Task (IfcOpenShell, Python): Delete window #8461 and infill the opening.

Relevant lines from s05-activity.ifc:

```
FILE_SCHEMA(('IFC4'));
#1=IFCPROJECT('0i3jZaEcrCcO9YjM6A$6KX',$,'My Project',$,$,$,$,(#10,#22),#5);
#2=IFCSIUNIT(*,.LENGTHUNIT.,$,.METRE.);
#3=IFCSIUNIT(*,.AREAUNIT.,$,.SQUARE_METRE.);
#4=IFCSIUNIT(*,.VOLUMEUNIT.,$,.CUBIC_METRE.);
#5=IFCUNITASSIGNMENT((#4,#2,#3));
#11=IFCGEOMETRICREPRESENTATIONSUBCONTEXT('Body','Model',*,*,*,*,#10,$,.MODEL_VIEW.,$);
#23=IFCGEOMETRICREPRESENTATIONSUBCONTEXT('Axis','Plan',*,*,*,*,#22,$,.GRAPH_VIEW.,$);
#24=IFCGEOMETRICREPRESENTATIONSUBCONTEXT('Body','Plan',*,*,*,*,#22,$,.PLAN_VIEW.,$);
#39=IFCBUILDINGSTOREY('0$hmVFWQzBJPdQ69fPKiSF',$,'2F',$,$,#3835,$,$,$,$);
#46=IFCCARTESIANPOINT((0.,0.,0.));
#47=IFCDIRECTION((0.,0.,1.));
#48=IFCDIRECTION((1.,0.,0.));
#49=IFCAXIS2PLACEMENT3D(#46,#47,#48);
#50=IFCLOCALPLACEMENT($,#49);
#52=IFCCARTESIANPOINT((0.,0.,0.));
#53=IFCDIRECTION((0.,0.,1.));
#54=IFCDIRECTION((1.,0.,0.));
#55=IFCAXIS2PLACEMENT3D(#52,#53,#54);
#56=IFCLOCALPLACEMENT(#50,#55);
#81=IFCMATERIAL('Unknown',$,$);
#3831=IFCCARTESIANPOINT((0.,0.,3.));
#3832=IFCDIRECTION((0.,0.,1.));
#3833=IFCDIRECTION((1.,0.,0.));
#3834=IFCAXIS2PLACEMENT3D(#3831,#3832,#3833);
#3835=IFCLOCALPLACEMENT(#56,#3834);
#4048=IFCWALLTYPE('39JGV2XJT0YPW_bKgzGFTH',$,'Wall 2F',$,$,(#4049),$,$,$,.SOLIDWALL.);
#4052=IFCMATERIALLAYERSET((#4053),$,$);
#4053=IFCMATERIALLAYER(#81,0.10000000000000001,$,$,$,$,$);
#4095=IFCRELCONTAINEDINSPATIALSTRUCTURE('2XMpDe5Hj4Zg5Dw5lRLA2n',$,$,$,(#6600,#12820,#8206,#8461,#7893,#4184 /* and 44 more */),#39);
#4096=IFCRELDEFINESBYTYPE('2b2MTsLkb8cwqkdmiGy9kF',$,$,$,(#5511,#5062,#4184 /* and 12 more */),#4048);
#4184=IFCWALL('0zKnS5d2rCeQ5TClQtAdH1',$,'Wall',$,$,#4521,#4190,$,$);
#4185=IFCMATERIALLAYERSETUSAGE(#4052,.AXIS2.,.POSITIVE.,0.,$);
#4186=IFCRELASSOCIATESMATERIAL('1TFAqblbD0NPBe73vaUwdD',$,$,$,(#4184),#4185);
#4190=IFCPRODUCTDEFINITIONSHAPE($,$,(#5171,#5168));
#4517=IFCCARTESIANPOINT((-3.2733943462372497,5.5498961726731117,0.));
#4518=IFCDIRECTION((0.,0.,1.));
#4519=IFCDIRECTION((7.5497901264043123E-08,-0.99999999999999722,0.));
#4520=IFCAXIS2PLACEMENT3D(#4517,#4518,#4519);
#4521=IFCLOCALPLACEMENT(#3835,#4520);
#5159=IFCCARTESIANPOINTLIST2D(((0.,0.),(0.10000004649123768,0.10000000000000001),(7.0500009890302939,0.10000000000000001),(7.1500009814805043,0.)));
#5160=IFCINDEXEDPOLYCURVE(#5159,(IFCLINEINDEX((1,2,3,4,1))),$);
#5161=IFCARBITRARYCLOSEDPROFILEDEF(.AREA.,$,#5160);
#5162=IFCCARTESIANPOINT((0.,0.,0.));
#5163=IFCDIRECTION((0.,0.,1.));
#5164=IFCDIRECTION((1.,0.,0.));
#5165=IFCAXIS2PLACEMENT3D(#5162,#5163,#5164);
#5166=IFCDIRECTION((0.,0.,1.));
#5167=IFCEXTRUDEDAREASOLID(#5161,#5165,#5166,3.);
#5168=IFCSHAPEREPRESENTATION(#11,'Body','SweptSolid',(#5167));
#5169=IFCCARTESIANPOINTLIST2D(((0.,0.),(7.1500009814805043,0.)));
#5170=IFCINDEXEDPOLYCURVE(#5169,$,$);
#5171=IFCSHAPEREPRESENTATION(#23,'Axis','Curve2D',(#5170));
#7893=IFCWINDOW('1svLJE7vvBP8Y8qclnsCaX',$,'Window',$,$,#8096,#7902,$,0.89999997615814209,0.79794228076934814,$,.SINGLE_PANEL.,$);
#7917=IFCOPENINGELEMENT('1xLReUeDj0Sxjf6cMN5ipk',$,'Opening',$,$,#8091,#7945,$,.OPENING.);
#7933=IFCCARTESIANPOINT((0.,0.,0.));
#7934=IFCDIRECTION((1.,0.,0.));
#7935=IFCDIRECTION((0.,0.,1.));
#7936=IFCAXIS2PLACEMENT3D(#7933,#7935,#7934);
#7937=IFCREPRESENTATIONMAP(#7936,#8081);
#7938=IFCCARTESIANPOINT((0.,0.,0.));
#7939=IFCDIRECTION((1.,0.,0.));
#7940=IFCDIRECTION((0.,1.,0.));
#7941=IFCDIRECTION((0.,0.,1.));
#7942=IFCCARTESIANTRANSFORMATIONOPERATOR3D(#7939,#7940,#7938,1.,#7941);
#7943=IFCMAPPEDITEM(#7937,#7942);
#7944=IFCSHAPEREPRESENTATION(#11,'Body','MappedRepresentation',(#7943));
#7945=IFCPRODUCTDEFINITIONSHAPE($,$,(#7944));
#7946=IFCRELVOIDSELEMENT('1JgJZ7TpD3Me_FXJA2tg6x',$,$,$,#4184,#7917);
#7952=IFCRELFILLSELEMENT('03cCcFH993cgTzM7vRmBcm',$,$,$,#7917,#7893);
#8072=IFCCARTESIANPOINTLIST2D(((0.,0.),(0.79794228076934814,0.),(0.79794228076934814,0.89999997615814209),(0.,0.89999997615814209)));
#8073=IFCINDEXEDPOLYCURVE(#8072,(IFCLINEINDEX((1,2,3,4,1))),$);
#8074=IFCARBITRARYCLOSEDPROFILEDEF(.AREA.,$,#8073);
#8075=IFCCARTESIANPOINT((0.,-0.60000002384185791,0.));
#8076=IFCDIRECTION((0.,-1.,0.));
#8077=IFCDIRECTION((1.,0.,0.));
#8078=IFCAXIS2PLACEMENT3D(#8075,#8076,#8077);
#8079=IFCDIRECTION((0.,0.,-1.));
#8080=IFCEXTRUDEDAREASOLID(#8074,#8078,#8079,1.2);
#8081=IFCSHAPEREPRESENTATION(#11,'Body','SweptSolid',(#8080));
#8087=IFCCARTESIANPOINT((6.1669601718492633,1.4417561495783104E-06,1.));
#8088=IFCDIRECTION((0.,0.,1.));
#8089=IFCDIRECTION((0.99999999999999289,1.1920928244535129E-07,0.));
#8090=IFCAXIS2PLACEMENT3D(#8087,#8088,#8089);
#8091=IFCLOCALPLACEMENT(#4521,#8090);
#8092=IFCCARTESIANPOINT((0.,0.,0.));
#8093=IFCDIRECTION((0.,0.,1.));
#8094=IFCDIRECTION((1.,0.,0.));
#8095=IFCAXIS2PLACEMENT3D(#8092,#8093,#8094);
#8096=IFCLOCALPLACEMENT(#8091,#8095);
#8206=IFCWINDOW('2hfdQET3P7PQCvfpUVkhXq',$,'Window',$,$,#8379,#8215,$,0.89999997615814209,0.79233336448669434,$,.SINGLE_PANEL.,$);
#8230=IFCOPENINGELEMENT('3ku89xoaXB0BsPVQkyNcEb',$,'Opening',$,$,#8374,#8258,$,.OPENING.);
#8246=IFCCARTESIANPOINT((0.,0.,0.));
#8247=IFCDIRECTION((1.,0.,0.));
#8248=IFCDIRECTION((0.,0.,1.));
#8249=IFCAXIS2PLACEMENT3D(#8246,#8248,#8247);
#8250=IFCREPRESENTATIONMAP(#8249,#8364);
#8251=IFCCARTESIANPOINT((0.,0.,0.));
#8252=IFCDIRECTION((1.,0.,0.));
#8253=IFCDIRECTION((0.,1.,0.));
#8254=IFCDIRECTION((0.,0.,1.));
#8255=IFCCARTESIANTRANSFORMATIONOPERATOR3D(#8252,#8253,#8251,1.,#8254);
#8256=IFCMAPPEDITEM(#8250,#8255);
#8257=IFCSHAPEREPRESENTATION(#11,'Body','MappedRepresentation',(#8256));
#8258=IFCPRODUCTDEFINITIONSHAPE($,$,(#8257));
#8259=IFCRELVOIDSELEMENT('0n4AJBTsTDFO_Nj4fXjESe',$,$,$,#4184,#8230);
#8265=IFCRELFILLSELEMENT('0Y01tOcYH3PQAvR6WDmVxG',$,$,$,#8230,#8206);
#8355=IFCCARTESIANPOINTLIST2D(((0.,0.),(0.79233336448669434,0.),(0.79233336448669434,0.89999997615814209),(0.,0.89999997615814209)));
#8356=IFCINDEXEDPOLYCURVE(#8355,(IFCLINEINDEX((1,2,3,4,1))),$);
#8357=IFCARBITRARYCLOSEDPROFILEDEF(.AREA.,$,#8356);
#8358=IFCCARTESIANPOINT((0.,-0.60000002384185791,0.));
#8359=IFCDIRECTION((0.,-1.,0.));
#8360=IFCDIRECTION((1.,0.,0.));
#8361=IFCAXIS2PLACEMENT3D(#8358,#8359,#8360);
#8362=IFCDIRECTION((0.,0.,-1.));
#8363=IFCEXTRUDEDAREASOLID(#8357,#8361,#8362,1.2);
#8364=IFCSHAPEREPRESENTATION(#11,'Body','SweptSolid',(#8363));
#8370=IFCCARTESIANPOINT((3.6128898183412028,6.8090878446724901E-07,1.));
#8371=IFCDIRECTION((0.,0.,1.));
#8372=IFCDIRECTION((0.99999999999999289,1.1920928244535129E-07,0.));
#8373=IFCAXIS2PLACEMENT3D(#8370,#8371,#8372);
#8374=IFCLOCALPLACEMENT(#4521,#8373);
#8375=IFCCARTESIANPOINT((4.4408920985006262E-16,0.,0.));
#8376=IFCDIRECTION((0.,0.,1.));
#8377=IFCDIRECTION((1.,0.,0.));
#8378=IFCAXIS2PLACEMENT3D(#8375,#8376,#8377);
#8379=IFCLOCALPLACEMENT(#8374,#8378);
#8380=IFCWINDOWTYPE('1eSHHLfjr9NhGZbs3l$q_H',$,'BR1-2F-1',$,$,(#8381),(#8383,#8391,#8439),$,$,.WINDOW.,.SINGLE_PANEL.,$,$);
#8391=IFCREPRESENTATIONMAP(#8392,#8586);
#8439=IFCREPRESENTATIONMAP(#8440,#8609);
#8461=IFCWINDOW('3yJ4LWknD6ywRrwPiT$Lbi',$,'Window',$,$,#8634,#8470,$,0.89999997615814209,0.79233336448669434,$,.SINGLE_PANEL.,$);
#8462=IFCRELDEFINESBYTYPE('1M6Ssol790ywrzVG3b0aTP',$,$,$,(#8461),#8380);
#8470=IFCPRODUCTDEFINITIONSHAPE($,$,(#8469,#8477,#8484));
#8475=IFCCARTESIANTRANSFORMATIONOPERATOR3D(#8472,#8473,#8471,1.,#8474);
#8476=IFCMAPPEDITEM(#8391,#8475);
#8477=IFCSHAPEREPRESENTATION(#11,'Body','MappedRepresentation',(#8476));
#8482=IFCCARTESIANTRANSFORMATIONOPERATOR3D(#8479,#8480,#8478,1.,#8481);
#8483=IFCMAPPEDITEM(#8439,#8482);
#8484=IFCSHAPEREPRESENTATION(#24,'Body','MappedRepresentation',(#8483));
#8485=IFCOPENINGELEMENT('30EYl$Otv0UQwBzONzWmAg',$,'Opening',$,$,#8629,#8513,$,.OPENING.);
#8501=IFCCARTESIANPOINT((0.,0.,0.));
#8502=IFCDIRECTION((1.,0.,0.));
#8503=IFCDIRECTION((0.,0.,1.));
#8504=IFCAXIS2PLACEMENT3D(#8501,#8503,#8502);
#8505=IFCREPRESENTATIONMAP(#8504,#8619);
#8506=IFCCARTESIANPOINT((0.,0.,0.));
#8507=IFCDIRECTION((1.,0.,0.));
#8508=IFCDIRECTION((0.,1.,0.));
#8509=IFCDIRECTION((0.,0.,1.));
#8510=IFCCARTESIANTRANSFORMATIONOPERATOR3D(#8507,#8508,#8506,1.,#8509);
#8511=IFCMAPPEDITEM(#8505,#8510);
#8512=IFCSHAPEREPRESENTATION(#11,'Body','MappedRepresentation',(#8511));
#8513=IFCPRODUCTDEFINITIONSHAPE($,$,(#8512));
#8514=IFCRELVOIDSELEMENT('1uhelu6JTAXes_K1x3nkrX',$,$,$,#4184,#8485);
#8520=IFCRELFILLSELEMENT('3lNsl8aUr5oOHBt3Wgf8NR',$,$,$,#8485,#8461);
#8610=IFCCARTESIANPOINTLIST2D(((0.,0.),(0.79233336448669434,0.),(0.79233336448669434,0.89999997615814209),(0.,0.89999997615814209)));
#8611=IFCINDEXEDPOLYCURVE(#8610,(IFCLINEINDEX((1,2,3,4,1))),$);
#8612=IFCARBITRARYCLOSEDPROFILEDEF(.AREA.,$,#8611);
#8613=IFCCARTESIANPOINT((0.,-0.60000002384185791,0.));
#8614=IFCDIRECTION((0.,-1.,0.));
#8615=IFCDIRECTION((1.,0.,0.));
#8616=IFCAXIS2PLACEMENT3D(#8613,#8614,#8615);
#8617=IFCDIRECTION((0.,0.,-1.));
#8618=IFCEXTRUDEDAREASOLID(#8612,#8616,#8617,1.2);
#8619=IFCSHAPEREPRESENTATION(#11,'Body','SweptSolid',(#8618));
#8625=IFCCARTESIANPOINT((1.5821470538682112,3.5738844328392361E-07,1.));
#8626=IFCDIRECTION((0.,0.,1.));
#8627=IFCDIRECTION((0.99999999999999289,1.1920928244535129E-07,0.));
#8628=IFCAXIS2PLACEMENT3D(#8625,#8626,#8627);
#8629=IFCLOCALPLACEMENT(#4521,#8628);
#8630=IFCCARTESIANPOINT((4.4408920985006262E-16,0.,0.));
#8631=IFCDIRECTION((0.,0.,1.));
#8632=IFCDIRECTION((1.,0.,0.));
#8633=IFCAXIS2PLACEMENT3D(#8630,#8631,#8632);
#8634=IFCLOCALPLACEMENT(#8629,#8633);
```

```python
import ifcopenshell
import ifcopenshell.api.feature
import ifcopenshell.api.root
import ifcopenshell.geom
import ifcopenshell.util.shape

model = ifcopenshell.open("s05-activity.ifc")
settings = ifcopenshell.geom.settings()


def volume(element):
    """Net volume in cubic metres, openings subtracted."""
    shape = ifcopenshell.geom.create_shape(settings, element)
    return ifcopenshell.util.shape.get_volume(shape.geometry)


window = model.by_id(8461)
opening = window.FillsVoids[0].RelatingOpeningElement
wall = opening.VoidsElements[0].RelatingBuildingElement
before = volume(wall)

ifcopenshell.api.root.remove_product(model, product=window)
ifcopenshell.api.feature.remove_feature(model, feature=opening)

after = volume(wall)

print(f"wall volume {before:.3f} -> {after:.3f} m3")

model.write("s05-activity_rev.ifc")
```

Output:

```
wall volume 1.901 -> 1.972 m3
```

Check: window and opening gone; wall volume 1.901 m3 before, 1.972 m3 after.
